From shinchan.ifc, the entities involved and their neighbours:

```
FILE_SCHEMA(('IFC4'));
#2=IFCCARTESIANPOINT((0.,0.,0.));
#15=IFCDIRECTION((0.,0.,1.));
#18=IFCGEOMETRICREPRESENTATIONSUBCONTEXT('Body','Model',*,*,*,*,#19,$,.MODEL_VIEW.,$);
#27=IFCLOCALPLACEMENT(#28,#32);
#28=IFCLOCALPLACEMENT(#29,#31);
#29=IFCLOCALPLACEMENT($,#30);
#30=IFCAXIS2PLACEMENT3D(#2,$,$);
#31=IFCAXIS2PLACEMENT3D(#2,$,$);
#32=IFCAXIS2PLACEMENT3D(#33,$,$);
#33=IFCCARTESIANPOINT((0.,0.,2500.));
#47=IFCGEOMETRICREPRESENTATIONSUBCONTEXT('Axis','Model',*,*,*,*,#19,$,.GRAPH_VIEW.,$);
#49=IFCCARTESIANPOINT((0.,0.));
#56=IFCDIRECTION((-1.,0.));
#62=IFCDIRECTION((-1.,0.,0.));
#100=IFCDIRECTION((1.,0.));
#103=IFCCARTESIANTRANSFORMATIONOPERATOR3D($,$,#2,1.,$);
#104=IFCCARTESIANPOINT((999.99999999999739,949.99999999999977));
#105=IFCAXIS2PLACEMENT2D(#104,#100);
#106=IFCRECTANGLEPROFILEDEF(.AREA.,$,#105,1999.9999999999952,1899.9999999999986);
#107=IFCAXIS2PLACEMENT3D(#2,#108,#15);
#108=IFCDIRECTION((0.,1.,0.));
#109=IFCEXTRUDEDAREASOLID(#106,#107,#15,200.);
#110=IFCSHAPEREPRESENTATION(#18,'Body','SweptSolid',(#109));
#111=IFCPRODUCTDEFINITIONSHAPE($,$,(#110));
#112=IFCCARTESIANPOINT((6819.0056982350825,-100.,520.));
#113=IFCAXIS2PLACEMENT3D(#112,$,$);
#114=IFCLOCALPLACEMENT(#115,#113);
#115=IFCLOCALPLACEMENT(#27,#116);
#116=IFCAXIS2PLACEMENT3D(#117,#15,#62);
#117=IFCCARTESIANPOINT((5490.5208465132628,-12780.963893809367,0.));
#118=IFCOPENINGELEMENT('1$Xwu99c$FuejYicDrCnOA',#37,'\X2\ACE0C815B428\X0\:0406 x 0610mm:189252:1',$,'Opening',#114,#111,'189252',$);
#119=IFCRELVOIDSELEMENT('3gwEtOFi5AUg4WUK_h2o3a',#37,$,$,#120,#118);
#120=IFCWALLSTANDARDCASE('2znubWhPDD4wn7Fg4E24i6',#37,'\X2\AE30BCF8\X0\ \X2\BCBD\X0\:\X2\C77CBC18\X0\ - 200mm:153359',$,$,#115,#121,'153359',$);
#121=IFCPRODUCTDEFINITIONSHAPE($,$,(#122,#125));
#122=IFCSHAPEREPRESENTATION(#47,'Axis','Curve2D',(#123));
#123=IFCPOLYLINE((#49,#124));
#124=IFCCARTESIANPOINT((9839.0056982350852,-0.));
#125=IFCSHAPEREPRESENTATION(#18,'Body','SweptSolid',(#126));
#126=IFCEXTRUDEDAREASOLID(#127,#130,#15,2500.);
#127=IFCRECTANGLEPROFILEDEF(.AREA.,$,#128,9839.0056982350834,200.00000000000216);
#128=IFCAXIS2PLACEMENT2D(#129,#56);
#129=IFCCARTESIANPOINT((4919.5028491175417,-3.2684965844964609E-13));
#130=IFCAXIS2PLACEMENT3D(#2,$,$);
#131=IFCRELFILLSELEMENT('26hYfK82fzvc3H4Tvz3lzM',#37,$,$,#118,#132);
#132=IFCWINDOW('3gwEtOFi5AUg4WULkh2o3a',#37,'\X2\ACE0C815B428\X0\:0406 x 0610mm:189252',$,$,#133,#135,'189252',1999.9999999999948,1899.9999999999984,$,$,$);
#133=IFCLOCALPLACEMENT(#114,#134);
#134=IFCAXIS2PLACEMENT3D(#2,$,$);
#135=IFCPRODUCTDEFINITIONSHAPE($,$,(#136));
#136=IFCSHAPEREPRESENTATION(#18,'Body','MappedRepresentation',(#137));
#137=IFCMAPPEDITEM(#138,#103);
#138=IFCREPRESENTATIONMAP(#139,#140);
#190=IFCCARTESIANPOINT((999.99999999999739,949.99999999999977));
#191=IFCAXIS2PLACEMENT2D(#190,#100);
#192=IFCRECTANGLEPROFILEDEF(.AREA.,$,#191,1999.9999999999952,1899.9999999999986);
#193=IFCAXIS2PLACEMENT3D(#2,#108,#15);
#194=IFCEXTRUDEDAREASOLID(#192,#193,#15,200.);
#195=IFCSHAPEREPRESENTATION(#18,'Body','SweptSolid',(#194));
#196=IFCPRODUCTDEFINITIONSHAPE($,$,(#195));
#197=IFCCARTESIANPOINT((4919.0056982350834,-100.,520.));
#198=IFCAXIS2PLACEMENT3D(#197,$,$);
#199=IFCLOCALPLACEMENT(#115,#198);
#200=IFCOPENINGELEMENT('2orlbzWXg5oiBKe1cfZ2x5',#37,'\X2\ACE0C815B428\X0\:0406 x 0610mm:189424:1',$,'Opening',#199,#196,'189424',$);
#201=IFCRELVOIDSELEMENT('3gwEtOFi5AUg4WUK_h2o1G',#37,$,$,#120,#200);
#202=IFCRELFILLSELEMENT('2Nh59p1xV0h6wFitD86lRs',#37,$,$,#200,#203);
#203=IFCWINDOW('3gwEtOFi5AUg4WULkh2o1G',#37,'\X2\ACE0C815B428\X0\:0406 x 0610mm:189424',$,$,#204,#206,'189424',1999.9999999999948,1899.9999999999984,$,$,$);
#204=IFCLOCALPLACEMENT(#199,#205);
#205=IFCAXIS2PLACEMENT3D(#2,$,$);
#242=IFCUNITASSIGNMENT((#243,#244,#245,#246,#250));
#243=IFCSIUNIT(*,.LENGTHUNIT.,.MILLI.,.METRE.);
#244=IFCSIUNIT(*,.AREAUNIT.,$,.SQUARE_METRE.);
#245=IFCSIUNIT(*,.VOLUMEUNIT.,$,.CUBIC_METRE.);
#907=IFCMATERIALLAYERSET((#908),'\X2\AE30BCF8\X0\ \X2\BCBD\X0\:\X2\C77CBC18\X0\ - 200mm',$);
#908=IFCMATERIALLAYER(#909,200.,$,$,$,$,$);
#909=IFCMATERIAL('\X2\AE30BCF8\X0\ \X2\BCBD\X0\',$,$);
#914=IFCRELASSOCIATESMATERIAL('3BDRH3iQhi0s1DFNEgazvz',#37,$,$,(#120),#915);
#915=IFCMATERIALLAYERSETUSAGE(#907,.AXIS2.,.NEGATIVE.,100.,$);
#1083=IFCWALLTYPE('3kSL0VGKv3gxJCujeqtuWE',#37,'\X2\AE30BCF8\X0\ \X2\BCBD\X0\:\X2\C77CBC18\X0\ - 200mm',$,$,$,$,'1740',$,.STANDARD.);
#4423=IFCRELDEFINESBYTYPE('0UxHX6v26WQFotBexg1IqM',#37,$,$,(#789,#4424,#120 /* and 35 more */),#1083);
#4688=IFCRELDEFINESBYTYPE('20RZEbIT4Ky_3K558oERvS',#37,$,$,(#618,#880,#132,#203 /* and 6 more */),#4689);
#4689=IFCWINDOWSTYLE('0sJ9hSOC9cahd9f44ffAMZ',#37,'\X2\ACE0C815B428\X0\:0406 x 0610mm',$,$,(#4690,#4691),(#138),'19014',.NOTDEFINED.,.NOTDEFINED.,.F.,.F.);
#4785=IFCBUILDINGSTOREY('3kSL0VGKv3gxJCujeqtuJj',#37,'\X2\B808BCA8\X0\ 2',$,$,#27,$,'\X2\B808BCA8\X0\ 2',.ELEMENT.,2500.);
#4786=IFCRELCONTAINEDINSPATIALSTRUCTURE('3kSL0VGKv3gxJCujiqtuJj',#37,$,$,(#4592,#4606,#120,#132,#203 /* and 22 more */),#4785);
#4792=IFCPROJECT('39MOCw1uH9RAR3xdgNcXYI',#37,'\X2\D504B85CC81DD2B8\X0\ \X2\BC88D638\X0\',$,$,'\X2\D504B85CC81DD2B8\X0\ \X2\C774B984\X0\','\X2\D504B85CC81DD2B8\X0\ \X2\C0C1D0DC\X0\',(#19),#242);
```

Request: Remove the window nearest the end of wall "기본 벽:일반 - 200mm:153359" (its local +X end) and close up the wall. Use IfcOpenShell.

```python
import ifcopenshell
import ifcopenshell.api.feature
import ifcopenshell.api.root
import ifcopenshell.geom
import ifcopenshell.util.shape

model = ifcopenshell.open("shinchan.ifc")
settings = ifcopenshell.geom.settings()


def volume(element):
    """Net volume in cubic metres, openings subtracted."""
    shape = ifcopenshell.geom.create_shape(settings, element)
    return ifcopenshell.util.shape.get_volume(shape.geometry)


window = model.by_id(132)
opening = window.FillsVoids[0].RelatingOpeningElement
wall = opening.VoidsElements[0].RelatingBuildingElement
before = volume(wall)

ifcopenshell.api.root.remove_product(model, product=window)
ifcopenshell.api.feature.remove_feature(model, feature=opening)

after = volume(wall)

print(f"wall volume {before:.3f} -> {after:.3f} m3")

model.write("shinchan_v2.ifc")
```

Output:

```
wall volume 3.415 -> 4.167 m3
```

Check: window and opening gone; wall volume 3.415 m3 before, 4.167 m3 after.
